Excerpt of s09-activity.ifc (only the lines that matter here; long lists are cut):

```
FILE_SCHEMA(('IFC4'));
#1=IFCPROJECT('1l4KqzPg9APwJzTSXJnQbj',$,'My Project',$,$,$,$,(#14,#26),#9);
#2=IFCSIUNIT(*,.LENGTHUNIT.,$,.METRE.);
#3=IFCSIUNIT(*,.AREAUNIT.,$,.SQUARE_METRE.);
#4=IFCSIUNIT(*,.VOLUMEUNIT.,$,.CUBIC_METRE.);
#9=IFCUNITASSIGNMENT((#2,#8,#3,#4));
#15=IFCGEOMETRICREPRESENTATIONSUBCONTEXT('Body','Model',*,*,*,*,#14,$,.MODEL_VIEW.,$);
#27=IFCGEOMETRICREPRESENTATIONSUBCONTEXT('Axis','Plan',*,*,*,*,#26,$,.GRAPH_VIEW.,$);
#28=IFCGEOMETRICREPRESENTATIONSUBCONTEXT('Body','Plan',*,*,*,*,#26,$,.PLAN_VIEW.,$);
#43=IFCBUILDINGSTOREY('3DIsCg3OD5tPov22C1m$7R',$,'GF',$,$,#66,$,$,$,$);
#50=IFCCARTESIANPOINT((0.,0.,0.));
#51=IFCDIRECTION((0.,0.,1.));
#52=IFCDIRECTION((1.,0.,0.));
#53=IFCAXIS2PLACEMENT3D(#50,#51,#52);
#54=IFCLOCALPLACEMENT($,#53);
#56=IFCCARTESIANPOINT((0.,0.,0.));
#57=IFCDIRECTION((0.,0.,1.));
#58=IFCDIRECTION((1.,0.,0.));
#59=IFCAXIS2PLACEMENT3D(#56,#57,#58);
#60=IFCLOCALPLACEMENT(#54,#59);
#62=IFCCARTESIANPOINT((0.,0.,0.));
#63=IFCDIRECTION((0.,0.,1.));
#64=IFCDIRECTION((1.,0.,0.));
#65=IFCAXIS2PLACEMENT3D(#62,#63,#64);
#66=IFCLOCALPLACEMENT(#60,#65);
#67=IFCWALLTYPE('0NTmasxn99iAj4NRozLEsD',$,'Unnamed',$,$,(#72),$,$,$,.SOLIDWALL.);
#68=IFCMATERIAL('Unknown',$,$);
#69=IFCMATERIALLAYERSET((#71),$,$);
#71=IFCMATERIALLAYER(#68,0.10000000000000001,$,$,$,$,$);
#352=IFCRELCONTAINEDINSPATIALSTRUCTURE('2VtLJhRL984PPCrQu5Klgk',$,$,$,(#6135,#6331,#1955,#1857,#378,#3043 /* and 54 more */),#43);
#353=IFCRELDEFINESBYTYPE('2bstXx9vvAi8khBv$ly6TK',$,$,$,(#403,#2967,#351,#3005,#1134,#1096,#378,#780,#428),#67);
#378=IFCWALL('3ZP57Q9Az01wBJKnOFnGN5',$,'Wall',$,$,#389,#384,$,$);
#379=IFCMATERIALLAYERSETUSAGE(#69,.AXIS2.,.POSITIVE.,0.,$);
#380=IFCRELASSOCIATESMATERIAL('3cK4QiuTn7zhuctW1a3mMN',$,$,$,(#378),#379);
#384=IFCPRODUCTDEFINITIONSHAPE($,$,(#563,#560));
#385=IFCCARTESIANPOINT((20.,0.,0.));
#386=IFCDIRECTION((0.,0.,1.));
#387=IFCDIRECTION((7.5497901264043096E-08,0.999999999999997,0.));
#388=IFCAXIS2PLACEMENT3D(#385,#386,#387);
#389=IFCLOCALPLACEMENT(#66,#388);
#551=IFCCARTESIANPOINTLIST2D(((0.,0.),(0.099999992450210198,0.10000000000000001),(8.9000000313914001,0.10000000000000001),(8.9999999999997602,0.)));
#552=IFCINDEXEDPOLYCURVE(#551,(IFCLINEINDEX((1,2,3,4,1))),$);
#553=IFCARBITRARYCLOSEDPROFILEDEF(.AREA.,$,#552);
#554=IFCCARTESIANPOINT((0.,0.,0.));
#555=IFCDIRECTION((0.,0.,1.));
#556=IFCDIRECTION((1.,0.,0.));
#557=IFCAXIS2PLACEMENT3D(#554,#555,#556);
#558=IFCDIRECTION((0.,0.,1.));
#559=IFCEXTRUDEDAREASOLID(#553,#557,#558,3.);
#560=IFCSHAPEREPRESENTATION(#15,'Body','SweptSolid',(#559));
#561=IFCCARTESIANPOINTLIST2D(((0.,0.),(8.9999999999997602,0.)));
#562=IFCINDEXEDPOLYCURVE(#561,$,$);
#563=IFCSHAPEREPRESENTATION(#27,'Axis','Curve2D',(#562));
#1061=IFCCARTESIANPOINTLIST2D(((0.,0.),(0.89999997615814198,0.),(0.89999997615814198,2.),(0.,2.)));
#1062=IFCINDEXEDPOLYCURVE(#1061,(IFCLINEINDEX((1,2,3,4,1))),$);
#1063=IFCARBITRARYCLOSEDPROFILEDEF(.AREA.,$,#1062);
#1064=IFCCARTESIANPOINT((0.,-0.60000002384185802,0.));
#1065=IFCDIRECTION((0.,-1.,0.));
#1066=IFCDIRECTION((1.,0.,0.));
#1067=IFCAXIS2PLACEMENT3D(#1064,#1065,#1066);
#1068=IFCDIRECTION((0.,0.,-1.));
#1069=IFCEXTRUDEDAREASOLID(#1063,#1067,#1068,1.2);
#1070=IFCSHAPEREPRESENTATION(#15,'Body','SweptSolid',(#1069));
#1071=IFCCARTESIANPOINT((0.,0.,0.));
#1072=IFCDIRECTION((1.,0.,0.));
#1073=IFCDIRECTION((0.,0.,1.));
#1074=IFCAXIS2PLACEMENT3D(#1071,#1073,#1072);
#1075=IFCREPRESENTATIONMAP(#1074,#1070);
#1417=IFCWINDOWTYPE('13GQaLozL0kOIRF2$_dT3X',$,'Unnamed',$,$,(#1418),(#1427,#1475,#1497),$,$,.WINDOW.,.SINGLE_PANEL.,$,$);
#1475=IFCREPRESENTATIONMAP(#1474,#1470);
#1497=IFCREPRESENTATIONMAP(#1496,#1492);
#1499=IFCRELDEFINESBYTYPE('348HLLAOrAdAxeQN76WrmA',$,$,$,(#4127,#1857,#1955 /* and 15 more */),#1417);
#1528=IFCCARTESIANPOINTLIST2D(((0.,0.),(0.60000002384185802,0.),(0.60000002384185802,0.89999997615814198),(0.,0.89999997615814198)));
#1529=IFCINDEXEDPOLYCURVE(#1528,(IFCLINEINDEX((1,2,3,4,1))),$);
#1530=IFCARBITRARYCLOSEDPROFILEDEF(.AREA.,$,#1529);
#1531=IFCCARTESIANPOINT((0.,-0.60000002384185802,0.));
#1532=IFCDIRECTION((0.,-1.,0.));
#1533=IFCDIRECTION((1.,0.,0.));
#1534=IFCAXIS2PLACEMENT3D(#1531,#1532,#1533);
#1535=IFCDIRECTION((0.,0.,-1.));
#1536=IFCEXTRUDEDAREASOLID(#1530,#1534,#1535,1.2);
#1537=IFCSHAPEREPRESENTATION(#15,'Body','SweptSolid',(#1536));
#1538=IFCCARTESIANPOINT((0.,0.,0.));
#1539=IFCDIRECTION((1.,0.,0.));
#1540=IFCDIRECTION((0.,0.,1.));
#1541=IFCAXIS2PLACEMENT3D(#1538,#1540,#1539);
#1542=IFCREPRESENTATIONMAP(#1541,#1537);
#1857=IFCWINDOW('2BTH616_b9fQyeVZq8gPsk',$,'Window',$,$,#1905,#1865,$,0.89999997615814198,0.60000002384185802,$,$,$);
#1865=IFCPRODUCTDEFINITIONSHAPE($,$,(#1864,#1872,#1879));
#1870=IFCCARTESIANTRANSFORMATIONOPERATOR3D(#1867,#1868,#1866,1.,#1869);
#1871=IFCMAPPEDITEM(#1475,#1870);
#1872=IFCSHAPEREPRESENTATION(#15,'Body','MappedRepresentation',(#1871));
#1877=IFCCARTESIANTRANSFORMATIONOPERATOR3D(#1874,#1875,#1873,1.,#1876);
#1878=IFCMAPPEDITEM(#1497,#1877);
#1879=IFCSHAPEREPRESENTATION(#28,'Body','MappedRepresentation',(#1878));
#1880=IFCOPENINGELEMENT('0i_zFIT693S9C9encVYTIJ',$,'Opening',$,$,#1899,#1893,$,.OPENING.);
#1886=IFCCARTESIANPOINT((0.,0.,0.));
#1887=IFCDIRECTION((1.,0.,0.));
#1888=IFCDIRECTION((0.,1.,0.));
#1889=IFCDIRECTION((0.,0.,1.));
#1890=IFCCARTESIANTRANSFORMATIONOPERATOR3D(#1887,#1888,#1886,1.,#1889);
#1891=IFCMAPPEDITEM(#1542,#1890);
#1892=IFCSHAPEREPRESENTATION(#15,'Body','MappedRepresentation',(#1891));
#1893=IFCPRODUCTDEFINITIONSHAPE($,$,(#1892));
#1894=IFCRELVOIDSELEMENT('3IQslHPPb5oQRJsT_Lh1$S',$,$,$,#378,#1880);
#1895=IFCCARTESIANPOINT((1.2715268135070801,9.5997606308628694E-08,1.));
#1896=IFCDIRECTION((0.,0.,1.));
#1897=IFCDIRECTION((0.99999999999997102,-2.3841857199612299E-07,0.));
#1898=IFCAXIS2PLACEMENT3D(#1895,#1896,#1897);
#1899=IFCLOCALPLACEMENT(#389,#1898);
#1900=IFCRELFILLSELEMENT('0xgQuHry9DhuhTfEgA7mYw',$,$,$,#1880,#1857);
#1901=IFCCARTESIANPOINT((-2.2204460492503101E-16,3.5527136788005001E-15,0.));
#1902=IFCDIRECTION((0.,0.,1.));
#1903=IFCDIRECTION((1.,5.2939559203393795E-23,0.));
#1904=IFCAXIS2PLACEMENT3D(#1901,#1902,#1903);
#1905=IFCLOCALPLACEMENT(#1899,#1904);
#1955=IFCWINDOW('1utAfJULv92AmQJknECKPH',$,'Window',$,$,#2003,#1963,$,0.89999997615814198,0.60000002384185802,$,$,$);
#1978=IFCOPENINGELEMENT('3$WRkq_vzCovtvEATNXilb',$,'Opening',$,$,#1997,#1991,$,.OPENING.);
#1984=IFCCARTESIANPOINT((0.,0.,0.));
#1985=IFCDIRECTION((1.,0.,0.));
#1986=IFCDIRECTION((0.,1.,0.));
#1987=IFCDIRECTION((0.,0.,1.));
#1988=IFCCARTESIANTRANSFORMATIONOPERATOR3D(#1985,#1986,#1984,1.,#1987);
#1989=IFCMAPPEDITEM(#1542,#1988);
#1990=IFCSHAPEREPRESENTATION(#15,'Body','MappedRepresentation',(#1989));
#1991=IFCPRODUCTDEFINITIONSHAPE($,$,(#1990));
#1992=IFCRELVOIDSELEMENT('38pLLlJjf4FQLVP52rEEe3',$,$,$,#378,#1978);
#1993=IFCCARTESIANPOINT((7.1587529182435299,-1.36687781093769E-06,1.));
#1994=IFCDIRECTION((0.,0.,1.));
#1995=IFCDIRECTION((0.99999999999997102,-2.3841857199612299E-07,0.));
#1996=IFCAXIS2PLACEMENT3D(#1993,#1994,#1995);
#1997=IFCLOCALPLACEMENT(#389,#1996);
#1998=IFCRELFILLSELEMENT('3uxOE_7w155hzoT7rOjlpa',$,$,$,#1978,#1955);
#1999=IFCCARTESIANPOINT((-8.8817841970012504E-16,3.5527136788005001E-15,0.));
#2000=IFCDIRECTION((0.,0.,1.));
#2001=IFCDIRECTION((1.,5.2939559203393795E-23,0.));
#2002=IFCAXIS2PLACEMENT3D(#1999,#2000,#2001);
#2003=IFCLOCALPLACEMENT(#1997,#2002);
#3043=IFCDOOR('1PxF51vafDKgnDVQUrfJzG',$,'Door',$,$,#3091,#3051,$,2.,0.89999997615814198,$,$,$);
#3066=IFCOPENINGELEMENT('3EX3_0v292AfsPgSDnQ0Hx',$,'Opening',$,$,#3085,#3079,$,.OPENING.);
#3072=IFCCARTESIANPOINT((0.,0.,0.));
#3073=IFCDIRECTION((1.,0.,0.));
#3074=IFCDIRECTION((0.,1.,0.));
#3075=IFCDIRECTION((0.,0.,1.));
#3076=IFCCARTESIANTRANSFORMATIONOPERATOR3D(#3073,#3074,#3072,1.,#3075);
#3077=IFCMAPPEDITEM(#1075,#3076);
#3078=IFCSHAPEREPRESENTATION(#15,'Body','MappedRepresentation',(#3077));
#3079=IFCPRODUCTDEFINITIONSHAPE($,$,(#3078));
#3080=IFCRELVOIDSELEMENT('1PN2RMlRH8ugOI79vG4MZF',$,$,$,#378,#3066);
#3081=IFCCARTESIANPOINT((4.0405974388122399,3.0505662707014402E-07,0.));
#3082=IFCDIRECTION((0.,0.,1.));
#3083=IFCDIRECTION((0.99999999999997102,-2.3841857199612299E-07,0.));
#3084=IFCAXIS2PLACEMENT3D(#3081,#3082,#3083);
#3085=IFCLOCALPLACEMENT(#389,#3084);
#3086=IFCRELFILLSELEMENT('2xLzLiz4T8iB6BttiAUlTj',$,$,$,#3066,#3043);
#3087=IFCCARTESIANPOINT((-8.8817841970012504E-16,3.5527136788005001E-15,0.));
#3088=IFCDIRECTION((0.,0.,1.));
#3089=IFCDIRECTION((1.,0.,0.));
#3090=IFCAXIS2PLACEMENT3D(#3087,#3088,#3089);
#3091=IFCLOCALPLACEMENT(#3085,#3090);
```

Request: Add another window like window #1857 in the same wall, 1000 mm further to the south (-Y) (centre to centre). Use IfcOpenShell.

```python
import ifcopenshell
import ifcopenshell.api.feature
import ifcopenshell.api.geometry
import ifcopenshell.api.root
import ifcopenshell.geom
import ifcopenshell.util.element
import ifcopenshell.util.placement
import ifcopenshell.util.shape

model = ifcopenshell.open("s09-activity.ifc")
settings = ifcopenshell.geom.settings()


def volume(element):
    """Net volume in cubic metres, openings subtracted."""
    shape = ifcopenshell.geom.create_shape(settings, element)
    return ifcopenshell.util.shape.get_volume(shape.geometry)


window = model.by_guid("2BTH616_b9fQyeVZq8gPsk")
opening = window.FillsVoids[0].RelatingOpeningElement
wall = opening.VoidsElements[0].RelatingBuildingElement
before = volume(wall)
shift = ifcopenshell.util.placement.get_local_placement(wall.ObjectPlacement)[:3, 0] * -1.0

# copy_class copies the void relationship, type, container and properties, but no geometry.
new_opening = ifcopenshell.api.root.copy_class(model, product=opening)
new_opening.Representation = ifcopenshell.util.element.copy_deep(
    model, opening.Representation, exclude=["IfcGeometricRepresentationContext", "IfcRepresentationMap"]
)
new_window = ifcopenshell.api.root.copy_class(model, product=window)
new_window.Representation = ifcopenshell.util.element.copy_deep(
    model, window.Representation, exclude=["IfcGeometricRepresentationContext", "IfcRepresentationMap"]
)
ifcopenshell.api.feature.add_filling(model, opening=new_opening, element=new_window)

for old, new in ((opening, new_opening), (window, new_window)):
    matrix = ifcopenshell.util.placement.get_local_placement(old.ObjectPlacement)
    matrix[:3, 3] += shift
    ifcopenshell.api.geometry.edit_object_placement(model, product=new, matrix=matrix, is_si=False)

after = volume(wall)

print(f"wall volume {before:.3f} -> {after:.3f} m3")

model.write("s09-activity-out.ifc")
```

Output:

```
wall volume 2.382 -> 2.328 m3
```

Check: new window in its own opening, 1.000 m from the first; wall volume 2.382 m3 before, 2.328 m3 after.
